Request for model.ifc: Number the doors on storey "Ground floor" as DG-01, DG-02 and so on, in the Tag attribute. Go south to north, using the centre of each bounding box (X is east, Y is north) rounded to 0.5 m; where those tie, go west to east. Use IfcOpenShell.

First a look at what the model holds.

```python
import ifcopenshell
import ifcopenshell.util.element
import ifcopenshell.util.placement

model = ifcopenshell.open("model.ifc")
print(model.schema)
storey = next(s for s in model.by_type("IfcBuildingStorey") if s.Name == "Ground floor")
doors = [e for e in ifcopenshell.util.element.get_decomposition(storey) if e.is_a("IfcDoor")]
for e in sorted(doors, key=lambda e: e.id()):
    origin = ifcopenshell.util.placement.get_local_placement(e.ObjectPlacement)[:3, 3]
    print(e.id(), e.Tag, e.Name, origin.round(2) + 0.0, sep=" | ")
```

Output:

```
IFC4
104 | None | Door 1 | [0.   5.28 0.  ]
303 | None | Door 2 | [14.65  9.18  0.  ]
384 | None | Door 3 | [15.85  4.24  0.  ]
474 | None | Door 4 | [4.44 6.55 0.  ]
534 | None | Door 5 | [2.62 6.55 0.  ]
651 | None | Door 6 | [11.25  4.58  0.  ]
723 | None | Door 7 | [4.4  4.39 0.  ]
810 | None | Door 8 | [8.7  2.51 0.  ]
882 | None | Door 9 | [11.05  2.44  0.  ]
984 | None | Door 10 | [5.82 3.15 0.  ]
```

```python
import ifcopenshell
import ifcopenshell.geom
import ifcopenshell.util.element
import ifcopenshell.util.shape

model = ifcopenshell.open("model.ifc")
settings = ifcopenshell.geom.settings()
settings.set("use-world-coords", True)


def centre(element):
    shape = ifcopenshell.geom.create_shape(settings, element)
    return ifcopenshell.util.shape.get_bbox_centroid(shape.geometry)


storey = next(s for s in model.by_type("IfcBuildingStorey") if s.Name == "Ground floor")
doors = [e for e in ifcopenshell.util.element.get_decomposition(storey) if e.is_a("IfcDoor")]

# Insertion points can sit at a corner or the storey origin, so sort by the geometry (in metres).
centres = {e: centre(e) for e in doors}
doors.sort(key=lambda e: (round(centres[e][1] / 0.5), centres[e][0]))

for i, e in enumerate(doors, start=1):
    number = f"DG-{i:02d}"
    e.Tag = number
    print(e.id(), number)

model.write("model_v2.ifc")
```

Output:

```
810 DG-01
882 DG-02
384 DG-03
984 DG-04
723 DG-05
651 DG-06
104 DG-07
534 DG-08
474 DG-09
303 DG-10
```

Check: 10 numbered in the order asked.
